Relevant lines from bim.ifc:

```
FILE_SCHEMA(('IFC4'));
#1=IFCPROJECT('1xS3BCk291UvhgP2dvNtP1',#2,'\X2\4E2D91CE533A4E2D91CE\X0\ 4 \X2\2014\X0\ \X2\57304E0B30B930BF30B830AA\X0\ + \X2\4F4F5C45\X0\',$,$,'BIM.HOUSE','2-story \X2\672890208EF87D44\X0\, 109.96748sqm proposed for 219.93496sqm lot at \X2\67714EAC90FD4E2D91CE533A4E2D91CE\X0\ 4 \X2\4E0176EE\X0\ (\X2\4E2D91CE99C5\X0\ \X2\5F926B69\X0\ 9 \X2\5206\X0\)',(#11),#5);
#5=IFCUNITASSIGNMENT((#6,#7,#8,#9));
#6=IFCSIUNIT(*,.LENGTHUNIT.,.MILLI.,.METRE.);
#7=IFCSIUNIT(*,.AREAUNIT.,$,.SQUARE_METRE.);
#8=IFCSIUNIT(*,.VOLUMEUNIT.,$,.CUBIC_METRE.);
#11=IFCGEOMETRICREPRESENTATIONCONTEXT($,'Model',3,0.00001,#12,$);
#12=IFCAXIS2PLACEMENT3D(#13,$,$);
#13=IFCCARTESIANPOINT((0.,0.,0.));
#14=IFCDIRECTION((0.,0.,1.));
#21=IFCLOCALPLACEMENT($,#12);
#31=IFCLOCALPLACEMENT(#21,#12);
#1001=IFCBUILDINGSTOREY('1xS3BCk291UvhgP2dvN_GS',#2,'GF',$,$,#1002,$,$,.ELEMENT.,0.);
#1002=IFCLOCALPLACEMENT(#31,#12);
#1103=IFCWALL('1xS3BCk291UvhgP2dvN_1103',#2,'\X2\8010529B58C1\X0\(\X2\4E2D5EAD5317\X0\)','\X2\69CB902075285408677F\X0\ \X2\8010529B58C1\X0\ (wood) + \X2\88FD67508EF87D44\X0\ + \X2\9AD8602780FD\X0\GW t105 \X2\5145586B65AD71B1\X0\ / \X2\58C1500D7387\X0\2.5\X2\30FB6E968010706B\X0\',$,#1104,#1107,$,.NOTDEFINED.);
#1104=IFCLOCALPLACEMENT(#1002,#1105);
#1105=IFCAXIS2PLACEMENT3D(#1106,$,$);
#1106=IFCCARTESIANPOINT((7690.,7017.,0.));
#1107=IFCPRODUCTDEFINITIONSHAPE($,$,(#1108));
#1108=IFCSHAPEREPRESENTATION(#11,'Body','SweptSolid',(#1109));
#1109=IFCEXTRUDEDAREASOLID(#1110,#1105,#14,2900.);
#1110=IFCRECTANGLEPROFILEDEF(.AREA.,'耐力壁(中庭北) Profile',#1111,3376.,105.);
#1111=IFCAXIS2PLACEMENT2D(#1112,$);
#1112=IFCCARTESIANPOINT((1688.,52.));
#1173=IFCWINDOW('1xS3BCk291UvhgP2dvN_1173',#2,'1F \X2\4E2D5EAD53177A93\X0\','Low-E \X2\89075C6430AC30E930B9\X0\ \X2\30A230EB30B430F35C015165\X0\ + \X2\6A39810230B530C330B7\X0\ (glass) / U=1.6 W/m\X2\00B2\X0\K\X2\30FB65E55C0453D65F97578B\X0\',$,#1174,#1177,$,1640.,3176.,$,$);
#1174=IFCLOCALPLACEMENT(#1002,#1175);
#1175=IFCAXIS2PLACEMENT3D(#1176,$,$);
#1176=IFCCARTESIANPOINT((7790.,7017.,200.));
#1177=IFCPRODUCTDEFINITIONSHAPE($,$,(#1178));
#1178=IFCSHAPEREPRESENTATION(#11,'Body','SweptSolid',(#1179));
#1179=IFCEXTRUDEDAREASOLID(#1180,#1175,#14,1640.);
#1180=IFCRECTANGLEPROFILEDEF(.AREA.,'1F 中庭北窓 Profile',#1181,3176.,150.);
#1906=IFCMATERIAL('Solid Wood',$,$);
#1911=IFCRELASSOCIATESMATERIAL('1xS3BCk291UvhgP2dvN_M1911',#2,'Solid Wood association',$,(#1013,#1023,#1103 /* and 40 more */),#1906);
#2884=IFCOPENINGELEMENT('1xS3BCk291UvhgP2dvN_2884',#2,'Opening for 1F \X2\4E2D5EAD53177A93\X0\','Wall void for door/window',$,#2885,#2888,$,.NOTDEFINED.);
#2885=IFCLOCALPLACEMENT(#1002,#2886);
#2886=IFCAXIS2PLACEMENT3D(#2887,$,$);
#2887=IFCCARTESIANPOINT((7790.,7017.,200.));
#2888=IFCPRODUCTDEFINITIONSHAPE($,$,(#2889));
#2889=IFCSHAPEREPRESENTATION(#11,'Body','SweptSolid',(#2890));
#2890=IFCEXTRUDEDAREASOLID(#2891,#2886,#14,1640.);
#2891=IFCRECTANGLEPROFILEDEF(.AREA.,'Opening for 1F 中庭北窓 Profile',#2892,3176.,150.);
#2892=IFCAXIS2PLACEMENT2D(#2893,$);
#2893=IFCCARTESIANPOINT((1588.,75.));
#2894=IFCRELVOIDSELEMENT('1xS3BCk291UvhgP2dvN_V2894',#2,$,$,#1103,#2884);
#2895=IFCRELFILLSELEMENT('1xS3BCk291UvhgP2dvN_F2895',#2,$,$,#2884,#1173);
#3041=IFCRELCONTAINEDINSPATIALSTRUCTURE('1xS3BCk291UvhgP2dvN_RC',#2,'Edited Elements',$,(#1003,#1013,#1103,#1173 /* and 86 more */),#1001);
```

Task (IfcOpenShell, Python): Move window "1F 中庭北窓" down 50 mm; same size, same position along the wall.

```python
import numpy as np
import ifcopenshell
import ifcopenshell.api.geometry
import ifcopenshell.util.placement
import ifcopenshell.util.unit

model = ifcopenshell.open("bim.ifc")
unit_scale = ifcopenshell.util.unit.calculate_unit_scale(model)

window = model.by_guid("1xS3BCk291UvhgP2dvN_1173")
opening = window.FillsVoids[0].RelatingOpeningElement
dz = -0.05 / unit_scale

shift = np.array([0.0, 0.0, dz])
# The window is not placed relative to its opening, so move both.
for product in (opening, window):
    matrix = ifcopenshell.util.placement.get_local_placement(product.ObjectPlacement)
    matrix[:3, 3] += shift
    ifcopenshell.api.geometry.edit_object_placement(model, product=product, matrix=matrix, is_si=False)

print(f"moved by {dz * unit_scale:+.3f} m")

model.write("bim_updated.ifc")
```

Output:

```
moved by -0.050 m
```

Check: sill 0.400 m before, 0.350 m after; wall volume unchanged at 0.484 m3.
